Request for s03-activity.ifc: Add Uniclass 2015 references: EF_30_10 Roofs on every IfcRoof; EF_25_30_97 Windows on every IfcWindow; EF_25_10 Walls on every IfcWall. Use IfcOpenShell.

First a look at what the model holds.

```python
import ifcopenshell

model = ifcopenshell.open("s03-activity.ifc")
print(model.schema)
print("classifications:", [c.Name for c in model.by_type("IfcClassification")])
for ifc_class in ("IfcDoor", "IfcRoof", "IfcStair", "IfcWall", "IfcWindow"):
    print(ifc_class, len(model.by_type(ifc_class)))
```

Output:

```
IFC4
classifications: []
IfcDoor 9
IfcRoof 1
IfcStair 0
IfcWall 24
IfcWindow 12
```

```python
import ifcopenshell
import ifcopenshell.api.classification

model = ifcopenshell.open("s03-activity.ifc")

system = ifcopenshell.api.classification.add_classification(model, classification="Uniclass 2015")

codes = {
    "IfcRoof": ("EF_30_10", "Roofs"),
    "IfcWindow": ("EF_25_30_97", "Windows"),
    "IfcWall": ("EF_25_10", "Walls"),
}
for ifc_class, (code, name) in codes.items():
    products = model.by_type(ifc_class)
    ifcopenshell.api.classification.add_reference(
        model, products=products, classification=system, identification=code, name=name
    )
    print(code, len(products))

model.write("s03-activity_v2.ifc")
```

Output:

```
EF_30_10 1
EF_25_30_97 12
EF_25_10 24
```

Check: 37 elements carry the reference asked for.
